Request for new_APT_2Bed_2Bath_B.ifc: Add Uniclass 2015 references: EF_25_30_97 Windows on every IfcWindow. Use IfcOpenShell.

First a look at what the model holds.

```python
import ifcopenshell

model = ifcopenshell.open("new_APT_2Bed_2Bath_B.ifc")
print(model.schema)
print("classifications:", [c.Name for c in model.by_type("IfcClassification")])
for ifc_class in ("IfcDoor", "IfcRoof", "IfcStair", "IfcWall", "IfcWindow"):
    print(ifc_class, len(model.by_type(ifc_class)))
```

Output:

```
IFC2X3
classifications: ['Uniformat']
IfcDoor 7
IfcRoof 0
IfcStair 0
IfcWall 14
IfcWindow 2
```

```python
import ifcopenshell
import ifcopenshell.api.classification

model = ifcopenshell.open("new_APT_2Bed_2Bath_B.ifc")

# IFC2X3 requires Source and Edition and has no link from the project to the system.
system = model.create_entity("IfcClassification", Source="NBS", Edition="2015", Name="Uniclass 2015")

codes = {
    "IfcWindow": ("EF_25_30_97", "Windows"),
}
for ifc_class, (code, name) in codes.items():
    products = model.by_type(ifc_class)
    ifcopenshell.api.classification.add_reference(
        model, products=products, classification=system, identification=code, name=name
    )
    print(code, len(products))

model.write("new_APT_2Bed_2Bath_B_updated.ifc")
```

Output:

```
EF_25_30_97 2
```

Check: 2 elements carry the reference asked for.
